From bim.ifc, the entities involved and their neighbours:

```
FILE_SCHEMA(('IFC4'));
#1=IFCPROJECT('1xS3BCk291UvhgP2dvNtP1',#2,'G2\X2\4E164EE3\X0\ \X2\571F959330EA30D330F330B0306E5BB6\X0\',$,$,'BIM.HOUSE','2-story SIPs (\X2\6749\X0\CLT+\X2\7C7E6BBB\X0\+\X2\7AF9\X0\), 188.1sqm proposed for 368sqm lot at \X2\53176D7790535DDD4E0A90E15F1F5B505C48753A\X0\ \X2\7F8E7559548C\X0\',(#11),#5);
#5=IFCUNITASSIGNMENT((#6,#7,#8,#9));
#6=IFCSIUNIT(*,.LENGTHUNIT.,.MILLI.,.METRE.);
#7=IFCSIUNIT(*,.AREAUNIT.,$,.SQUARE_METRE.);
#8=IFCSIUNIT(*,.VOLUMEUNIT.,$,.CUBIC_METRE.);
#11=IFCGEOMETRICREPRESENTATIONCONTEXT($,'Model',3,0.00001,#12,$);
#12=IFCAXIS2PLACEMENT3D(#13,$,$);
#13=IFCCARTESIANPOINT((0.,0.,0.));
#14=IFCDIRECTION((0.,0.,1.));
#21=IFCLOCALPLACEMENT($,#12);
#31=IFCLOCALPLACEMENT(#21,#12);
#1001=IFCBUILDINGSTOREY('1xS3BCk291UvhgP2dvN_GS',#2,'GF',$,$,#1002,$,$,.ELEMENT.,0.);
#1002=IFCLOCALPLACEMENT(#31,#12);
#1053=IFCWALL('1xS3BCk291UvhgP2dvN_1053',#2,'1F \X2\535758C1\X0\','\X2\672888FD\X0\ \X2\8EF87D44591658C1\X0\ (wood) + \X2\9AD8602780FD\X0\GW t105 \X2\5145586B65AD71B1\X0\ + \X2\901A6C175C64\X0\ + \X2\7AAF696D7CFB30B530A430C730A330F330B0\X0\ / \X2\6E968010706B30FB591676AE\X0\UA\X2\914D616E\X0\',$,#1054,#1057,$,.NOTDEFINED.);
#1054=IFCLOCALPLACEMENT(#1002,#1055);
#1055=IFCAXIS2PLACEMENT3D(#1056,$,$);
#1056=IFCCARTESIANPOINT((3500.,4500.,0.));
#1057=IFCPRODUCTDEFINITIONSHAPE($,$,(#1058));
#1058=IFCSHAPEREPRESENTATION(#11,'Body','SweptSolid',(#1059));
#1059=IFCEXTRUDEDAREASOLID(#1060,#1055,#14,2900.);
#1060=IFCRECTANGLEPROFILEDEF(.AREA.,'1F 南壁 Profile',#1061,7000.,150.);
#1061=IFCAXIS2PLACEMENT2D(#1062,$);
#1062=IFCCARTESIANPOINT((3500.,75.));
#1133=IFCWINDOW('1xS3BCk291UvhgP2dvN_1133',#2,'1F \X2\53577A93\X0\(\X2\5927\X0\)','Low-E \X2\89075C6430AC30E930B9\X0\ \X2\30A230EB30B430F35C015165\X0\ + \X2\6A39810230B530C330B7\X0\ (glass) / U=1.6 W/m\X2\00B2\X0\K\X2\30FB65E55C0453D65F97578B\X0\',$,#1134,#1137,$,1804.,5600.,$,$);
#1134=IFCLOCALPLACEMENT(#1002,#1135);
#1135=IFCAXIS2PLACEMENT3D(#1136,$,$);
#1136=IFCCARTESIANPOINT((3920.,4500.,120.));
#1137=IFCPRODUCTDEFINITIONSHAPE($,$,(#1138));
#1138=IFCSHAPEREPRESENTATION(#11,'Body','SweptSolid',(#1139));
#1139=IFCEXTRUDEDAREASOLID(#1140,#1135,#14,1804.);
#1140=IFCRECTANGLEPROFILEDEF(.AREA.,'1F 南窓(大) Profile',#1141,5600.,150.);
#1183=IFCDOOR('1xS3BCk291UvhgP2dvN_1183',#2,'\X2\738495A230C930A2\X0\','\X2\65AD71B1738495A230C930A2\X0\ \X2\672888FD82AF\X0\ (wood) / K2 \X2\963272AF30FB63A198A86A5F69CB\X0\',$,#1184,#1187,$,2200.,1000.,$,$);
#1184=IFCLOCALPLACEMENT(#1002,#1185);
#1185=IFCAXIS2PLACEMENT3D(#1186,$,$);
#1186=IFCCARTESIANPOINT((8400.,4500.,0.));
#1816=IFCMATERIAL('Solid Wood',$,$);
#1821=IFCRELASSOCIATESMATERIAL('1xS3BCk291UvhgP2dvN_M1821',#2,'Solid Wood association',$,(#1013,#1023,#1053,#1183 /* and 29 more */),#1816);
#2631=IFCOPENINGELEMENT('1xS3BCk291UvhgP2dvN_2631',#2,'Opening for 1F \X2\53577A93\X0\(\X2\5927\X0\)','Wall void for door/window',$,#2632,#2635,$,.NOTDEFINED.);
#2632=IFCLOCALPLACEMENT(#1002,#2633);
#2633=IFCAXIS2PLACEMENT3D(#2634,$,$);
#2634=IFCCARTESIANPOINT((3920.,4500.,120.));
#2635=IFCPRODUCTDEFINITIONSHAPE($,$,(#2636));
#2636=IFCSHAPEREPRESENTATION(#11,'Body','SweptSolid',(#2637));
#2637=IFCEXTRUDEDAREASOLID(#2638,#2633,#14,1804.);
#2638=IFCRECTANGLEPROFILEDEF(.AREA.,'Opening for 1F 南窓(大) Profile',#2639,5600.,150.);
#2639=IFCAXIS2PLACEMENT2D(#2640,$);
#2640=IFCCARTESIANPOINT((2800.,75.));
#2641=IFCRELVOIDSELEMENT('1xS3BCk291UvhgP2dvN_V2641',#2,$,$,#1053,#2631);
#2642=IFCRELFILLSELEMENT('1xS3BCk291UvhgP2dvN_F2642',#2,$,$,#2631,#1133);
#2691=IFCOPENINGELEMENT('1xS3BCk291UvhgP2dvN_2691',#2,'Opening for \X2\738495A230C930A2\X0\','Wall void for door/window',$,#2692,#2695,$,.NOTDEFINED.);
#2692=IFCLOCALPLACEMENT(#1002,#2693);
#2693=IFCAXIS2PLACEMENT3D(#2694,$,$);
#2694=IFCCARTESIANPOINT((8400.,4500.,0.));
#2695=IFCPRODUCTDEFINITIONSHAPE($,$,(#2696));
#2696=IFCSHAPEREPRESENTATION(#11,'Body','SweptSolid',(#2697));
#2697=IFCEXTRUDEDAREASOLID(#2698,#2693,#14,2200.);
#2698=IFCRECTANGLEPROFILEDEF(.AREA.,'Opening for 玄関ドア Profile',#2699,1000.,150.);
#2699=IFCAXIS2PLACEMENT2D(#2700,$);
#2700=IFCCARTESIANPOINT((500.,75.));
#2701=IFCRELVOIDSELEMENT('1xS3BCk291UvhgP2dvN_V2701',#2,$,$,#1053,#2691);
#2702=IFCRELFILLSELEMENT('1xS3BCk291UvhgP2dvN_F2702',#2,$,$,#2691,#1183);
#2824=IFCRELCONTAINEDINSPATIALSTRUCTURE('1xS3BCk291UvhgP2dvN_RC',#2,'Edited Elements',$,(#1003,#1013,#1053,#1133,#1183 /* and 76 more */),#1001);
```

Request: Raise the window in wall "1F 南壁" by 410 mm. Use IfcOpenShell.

```python
import numpy as np
import ifcopenshell
import ifcopenshell.api.geometry
import ifcopenshell.util.placement
import ifcopenshell.util.unit

model = ifcopenshell.open("bim.ifc")
unit_scale = ifcopenshell.util.unit.calculate_unit_scale(model)

window = model.by_id(1133)
opening = window.FillsVoids[0].RelatingOpeningElement
dz = 0.41 / unit_scale

shift = np.array([0.0, 0.0, dz])
# The window is not placed relative to its opening, so move both.
for product in (opening, window):
    matrix = ifcopenshell.util.placement.get_local_placement(product.ObjectPlacement)
    matrix[:3, 3] += shift
    ifcopenshell.api.geometry.edit_object_placement(model, product=product, matrix=matrix, is_si=False)

print(f"moved by {dz * unit_scale:+.3f} m")

model.write("bim_rev.ifc")
```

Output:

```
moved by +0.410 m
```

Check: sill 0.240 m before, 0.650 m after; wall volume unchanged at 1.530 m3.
